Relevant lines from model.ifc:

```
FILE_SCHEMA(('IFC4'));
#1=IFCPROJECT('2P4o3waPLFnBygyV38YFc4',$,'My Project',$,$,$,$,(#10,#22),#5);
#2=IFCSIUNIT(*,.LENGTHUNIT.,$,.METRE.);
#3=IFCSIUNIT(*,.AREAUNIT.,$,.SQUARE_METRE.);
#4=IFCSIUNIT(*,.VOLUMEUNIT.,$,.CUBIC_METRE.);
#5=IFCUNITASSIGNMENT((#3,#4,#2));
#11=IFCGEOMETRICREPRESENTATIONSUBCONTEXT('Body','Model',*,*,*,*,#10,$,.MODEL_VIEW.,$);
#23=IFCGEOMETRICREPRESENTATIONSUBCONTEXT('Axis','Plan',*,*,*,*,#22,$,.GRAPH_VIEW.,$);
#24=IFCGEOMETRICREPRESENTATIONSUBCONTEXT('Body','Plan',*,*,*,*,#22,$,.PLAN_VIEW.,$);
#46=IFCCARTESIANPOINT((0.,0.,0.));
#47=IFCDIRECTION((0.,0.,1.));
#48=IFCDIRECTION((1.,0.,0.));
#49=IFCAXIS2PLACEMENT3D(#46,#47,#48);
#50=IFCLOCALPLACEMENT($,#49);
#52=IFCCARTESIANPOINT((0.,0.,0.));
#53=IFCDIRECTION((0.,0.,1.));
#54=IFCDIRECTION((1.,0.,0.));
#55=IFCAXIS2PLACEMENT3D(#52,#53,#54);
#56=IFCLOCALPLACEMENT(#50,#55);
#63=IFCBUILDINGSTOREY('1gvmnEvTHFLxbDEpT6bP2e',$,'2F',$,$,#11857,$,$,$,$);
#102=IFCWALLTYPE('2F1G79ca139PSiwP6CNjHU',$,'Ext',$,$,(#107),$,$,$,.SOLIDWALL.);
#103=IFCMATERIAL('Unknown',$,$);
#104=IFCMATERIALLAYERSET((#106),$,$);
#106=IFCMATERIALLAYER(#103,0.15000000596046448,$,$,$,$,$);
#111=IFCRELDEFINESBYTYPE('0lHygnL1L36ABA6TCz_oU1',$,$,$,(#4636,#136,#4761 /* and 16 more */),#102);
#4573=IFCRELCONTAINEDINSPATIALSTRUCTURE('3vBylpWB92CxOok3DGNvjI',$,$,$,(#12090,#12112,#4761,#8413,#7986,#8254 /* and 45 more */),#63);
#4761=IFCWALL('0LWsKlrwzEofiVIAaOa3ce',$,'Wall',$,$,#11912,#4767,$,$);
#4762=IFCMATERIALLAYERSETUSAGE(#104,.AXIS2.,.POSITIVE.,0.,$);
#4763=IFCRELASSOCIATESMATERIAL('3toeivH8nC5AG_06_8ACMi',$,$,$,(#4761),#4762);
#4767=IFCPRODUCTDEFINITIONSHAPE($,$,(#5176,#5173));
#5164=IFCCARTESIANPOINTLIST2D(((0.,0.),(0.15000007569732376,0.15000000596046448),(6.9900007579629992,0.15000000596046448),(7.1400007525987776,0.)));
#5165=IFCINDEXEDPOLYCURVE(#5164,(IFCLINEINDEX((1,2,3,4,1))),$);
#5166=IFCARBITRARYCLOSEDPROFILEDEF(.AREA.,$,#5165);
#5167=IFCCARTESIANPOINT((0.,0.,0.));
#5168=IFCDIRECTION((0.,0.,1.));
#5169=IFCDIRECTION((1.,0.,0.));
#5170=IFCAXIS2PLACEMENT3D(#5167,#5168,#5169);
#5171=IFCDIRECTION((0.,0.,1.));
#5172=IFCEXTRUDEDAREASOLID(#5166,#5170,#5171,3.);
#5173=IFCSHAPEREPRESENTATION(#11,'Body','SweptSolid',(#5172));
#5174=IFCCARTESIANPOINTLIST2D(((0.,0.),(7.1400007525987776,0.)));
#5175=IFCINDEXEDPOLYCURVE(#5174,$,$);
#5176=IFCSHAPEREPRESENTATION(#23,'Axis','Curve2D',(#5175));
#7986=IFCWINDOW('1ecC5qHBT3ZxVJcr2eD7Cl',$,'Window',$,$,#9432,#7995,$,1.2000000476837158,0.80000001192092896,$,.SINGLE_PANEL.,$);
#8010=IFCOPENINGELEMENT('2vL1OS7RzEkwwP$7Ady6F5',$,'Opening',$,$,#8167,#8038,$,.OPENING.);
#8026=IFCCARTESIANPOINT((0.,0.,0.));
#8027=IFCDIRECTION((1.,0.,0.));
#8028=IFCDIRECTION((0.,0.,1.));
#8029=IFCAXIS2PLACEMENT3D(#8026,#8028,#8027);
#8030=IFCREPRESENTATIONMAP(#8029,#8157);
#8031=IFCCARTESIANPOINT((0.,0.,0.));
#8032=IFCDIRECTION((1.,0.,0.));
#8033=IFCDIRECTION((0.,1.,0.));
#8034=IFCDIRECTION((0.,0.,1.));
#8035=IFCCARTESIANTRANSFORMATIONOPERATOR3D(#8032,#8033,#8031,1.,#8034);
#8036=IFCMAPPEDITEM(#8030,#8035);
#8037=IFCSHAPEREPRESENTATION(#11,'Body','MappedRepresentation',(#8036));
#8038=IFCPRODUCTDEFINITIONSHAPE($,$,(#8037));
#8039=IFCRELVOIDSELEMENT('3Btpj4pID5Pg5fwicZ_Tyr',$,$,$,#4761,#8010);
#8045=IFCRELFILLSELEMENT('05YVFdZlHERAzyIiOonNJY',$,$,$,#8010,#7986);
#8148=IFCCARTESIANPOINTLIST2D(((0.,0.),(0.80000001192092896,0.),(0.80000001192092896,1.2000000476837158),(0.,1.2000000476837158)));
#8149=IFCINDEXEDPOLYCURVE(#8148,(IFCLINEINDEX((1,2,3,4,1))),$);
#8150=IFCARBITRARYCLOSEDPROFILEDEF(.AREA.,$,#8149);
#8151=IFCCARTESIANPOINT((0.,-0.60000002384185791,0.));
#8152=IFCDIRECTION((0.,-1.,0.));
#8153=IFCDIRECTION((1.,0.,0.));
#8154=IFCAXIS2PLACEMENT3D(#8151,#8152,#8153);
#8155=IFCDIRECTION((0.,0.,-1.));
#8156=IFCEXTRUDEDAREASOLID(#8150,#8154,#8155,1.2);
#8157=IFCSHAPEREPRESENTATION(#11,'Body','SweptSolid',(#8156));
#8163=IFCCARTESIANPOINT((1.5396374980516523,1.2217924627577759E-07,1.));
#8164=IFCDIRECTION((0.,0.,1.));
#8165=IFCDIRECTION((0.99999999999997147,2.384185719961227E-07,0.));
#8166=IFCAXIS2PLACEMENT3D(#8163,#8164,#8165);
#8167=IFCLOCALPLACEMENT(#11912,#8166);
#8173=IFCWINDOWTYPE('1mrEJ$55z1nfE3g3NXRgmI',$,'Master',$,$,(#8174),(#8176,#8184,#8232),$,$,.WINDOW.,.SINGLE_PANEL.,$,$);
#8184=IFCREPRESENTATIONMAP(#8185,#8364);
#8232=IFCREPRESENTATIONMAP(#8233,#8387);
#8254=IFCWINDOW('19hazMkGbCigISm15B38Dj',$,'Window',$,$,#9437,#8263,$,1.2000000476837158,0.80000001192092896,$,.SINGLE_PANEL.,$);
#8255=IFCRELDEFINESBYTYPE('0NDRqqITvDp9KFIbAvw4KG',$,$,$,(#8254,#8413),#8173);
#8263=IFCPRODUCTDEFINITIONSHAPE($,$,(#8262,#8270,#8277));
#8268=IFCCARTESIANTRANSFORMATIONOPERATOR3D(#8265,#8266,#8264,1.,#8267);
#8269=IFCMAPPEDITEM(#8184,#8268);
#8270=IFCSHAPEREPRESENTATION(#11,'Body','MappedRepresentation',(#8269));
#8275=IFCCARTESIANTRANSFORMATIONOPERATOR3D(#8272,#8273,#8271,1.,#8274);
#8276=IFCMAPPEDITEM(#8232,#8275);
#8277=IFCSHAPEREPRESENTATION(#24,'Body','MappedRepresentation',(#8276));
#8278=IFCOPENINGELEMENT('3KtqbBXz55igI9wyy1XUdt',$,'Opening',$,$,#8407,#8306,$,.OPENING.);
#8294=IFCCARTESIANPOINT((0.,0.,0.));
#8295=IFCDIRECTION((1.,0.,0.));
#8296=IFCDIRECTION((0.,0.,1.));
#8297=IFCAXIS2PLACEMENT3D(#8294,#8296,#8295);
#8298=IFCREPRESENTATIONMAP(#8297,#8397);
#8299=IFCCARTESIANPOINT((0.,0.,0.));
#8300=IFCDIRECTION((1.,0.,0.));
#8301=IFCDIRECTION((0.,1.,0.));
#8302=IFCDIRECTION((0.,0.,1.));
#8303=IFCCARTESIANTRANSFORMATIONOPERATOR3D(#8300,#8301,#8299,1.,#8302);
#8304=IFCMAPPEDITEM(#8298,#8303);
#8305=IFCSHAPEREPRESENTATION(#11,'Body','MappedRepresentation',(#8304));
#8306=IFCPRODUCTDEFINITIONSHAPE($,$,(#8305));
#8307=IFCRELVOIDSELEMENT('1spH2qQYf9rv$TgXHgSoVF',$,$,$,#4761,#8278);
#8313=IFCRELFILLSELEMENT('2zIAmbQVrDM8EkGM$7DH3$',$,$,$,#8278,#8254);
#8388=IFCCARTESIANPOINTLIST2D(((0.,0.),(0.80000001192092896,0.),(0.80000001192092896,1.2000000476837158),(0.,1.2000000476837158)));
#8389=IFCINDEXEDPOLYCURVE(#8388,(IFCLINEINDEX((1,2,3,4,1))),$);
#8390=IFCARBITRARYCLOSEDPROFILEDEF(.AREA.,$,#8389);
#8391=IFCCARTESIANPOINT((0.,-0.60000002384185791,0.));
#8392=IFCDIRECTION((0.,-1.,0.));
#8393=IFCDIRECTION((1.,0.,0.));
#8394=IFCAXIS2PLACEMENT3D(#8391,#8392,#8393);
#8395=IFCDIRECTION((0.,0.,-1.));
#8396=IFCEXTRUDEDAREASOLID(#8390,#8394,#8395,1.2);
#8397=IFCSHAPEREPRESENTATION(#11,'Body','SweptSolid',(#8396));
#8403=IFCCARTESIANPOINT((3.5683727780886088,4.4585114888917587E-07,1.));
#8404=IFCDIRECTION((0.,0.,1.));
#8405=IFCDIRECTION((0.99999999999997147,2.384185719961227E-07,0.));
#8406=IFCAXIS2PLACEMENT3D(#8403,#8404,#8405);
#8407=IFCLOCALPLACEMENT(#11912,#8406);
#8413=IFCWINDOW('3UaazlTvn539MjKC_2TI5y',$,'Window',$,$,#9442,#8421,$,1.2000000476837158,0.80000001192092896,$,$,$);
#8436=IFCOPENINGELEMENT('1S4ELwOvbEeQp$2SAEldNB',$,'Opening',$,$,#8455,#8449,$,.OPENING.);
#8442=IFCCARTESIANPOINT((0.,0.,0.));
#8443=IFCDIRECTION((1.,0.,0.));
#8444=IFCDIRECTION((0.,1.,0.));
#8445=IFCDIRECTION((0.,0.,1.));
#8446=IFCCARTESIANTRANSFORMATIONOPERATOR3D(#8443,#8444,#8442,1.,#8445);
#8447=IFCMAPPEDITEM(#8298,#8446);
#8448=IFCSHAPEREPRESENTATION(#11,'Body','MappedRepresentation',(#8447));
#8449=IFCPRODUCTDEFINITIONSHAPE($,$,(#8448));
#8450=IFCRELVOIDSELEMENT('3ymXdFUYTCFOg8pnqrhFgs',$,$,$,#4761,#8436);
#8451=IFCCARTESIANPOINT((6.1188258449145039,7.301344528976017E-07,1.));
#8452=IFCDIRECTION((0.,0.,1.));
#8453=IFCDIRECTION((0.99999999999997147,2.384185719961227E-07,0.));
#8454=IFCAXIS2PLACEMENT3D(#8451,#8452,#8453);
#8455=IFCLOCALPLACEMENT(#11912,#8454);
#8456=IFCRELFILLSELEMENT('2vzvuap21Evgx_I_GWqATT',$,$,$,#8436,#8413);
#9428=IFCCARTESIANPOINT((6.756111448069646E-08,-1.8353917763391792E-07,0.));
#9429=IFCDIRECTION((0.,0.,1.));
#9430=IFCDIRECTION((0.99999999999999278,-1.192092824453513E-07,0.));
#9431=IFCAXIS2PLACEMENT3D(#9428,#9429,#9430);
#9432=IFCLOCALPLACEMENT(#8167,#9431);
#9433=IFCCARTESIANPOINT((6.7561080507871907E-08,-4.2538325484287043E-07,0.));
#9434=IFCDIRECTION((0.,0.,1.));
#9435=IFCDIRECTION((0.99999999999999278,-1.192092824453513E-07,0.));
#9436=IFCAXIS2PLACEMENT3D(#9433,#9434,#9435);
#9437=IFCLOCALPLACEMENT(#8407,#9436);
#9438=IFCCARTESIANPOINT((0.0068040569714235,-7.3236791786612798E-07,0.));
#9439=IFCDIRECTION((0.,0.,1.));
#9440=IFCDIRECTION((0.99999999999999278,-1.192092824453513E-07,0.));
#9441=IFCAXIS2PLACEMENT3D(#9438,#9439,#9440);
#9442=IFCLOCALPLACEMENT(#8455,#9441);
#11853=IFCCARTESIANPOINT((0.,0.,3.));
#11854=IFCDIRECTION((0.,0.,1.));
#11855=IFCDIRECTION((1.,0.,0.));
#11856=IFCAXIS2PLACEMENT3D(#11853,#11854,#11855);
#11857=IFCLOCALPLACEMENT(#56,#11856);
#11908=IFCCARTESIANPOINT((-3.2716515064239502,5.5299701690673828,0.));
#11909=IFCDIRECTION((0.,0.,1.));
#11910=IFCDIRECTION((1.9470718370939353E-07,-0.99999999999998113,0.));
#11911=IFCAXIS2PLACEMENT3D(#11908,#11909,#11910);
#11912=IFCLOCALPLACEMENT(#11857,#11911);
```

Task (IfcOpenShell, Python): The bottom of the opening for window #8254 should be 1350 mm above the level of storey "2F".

```python
import numpy as np
import ifcopenshell
import ifcopenshell.api.geometry
import ifcopenshell.geom
import ifcopenshell.util.element
import ifcopenshell.util.placement
import ifcopenshell.util.shape
import ifcopenshell.util.unit

model = ifcopenshell.open("model.ifc")
unit_scale = ifcopenshell.util.unit.calculate_unit_scale(model)

window = model.by_guid("19hazMkGbCigISm15B38Dj")
opening = window.FillsVoids[0].RelatingOpeningElement
storey = ifcopenshell.util.element.get_container(window, ifc_class="IfcBuildingStorey")
level = ifcopenshell.util.placement.get_local_placement(storey.ObjectPlacement)[2, 3]

# The opening's origin need not be at the sill, so measure its lowest point.
shape = ifcopenshell.geom.create_shape(ifcopenshell.geom.settings(), opening)
bottom = ifcopenshell.util.shape.get_shape_bottom_elevation(shape, shape.geometry) / unit_scale
dz = level + 1.35 - bottom

shift = np.array([0.0, 0.0, dz])
# The window is placed relative to its opening, so it follows when the opening moves.
matrix = ifcopenshell.util.placement.get_local_placement(opening.ObjectPlacement)
matrix[:3, 3] += shift
ifcopenshell.api.geometry.edit_object_placement(
    model, product=opening, matrix=matrix, is_si=False, should_transform_children=True
)

print(f"moved by {dz * unit_scale:+.3f} m")

model.write("model_updated.ifc")
```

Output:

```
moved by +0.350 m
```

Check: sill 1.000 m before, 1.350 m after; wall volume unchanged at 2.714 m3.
